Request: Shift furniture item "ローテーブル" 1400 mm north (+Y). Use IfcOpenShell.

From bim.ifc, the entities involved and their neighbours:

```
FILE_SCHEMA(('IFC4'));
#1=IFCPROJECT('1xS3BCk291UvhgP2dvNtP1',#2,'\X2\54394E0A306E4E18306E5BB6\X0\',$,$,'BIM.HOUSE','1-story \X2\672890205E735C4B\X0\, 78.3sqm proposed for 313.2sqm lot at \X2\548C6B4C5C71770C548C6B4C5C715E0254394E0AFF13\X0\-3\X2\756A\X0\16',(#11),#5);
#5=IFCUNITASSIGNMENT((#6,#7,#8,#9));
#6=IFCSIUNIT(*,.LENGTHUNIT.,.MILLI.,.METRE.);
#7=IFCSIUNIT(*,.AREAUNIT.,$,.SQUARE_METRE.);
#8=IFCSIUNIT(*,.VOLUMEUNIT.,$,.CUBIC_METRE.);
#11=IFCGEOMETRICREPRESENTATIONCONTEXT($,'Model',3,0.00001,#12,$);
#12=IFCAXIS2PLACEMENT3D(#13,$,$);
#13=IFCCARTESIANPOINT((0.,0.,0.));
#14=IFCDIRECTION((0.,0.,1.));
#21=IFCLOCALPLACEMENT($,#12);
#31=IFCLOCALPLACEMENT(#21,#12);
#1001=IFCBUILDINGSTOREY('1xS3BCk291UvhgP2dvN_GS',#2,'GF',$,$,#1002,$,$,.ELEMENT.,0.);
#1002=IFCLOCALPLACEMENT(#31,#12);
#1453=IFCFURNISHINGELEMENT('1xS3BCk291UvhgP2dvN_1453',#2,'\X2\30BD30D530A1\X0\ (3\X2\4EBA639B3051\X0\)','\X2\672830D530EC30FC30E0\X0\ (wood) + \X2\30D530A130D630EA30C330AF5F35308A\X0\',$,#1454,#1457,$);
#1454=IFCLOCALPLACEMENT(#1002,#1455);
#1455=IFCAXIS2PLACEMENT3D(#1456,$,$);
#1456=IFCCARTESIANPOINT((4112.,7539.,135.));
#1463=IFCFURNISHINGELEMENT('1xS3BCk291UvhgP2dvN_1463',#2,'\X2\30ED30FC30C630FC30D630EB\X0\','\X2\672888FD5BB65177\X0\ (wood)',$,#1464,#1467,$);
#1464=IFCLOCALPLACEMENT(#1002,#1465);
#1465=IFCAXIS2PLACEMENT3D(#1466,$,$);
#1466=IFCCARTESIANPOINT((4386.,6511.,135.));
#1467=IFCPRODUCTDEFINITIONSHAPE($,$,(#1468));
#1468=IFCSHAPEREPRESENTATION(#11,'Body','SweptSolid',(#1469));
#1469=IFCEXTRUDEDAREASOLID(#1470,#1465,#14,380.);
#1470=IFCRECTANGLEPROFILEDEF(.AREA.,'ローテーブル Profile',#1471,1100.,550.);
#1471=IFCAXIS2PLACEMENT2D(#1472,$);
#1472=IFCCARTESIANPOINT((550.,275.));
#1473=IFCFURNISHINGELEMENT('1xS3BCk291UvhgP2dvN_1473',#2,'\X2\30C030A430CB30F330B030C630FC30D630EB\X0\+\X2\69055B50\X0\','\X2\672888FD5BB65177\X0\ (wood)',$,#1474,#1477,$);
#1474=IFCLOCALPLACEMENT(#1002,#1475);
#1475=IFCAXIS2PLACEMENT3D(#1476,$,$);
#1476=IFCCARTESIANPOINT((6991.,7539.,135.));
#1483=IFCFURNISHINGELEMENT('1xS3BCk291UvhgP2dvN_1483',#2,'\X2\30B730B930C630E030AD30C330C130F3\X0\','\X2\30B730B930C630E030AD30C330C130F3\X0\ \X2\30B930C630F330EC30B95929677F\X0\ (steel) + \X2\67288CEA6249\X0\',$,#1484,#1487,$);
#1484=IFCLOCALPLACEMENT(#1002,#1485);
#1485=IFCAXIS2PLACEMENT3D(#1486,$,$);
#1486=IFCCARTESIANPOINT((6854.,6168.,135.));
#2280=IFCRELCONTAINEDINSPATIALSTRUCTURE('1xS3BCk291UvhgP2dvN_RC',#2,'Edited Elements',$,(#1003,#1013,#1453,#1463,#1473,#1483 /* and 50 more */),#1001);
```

```python
import ifcopenshell
import ifcopenshell.api.geometry
import ifcopenshell.util.placement
import ifcopenshell.util.unit

model = ifcopenshell.open("bim.ifc")
unit_scale = ifcopenshell.util.unit.calculate_unit_scale(model)

item = model.by_id(1463)
matrix = ifcopenshell.util.placement.get_local_placement(item.ObjectPlacement)
matrix[1, 3] += 1.4 / unit_scale
ifcopenshell.api.geometry.edit_object_placement(model, product=item, matrix=matrix, is_si=False)

print(ifcopenshell.util.placement.get_local_placement(item.ObjectPlacement).round(3) + 0.0)

model.write("bim-out.ifc")
```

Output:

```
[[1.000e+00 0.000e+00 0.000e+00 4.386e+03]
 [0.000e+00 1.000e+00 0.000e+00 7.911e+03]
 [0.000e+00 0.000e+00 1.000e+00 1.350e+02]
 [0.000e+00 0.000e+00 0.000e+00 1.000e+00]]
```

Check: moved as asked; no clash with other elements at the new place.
